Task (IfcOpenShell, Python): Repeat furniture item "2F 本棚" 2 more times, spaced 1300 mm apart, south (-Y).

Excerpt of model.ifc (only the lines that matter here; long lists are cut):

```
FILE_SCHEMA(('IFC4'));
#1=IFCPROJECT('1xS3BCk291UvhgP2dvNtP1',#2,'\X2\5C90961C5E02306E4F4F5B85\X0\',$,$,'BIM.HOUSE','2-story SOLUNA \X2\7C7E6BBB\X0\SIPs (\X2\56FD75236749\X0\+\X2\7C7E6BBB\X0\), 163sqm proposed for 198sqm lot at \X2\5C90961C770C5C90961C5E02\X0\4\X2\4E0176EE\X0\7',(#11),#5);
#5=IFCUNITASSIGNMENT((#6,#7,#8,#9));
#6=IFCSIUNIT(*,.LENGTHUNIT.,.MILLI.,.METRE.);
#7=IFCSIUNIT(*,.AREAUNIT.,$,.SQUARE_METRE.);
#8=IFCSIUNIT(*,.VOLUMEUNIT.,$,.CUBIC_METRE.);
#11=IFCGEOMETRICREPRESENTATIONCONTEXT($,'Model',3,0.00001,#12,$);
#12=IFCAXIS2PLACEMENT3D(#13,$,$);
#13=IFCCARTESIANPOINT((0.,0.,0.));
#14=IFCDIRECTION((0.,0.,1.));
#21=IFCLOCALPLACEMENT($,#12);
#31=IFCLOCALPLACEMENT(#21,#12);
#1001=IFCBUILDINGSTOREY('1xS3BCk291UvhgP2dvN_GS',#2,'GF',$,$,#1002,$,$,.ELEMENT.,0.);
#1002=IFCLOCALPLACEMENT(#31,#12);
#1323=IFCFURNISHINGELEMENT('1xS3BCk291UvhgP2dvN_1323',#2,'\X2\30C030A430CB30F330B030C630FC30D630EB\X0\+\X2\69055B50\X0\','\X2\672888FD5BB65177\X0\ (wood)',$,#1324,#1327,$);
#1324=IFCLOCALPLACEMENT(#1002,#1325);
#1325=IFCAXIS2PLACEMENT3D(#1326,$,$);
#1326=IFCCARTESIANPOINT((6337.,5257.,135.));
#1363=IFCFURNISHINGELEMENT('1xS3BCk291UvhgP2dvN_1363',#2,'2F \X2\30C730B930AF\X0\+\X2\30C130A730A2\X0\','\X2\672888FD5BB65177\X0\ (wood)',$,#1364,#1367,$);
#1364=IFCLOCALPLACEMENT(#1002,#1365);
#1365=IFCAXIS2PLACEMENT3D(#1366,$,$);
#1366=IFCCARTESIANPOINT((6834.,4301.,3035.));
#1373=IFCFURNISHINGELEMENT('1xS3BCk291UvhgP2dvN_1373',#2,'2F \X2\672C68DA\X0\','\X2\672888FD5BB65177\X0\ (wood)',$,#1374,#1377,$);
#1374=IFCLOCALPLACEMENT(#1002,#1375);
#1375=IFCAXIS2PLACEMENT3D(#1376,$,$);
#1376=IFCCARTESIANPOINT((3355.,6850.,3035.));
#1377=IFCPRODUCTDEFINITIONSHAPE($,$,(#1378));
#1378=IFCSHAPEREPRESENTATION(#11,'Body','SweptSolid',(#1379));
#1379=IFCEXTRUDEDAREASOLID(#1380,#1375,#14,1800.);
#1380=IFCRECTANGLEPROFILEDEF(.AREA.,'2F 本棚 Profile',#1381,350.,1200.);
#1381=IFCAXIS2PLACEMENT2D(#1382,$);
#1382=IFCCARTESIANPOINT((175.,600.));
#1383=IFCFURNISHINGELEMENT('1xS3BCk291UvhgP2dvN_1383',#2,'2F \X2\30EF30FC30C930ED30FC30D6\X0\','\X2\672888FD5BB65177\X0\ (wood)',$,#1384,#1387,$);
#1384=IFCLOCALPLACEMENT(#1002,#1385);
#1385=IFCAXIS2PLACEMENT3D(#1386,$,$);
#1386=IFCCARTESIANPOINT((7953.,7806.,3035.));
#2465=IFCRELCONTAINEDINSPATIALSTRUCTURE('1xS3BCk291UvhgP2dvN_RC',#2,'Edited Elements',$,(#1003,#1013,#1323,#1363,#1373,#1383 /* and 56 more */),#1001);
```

```python
import numpy as np
import ifcopenshell
import ifcopenshell.api.geometry
import ifcopenshell.api.root
import ifcopenshell.util.element
import ifcopenshell.util.placement
import ifcopenshell.util.unit

model = ifcopenshell.open("model.ifc")
unit_scale = ifcopenshell.util.unit.calculate_unit_scale(model)


def reuse_history(source, copy):
    """copy_class also copies each property set's owner history, people and application; keep the originals."""
    for rel in copy.IsDefinedBy:
        if rel.is_a("IfcRelDefinesByProperties") and (history := rel.RelatingPropertyDefinition.OwnerHistory):
            rel.RelatingPropertyDefinition.OwnerHistory = source.OwnerHistory
            ifcopenshell.util.element.remove_deep2(model, history)


source = model.by_guid("1xS3BCk291UvhgP2dvN_1373")
base = ifcopenshell.util.placement.get_local_placement(source.ObjectPlacement)
step = np.array([0.0, -1.0, 0.0]) * 1.3 / unit_scale

for i in range(1, 3):
    copy = ifcopenshell.api.root.copy_class(model, product=source)
    copy.Representation = ifcopenshell.util.element.copy_deep(
        model, source.Representation, exclude=["IfcGeometricRepresentationContext", "IfcRepresentationMap"]
    )
    reuse_history(source, copy)
    matrix = base.copy()
    matrix[:3, 3] += i * step
    print("added at", matrix[:3, 3].round(3) + 0.0)
    ifcopenshell.api.geometry.edit_object_placement(model, product=copy, matrix=matrix, is_si=False)

model.write("model_updated.ifc")
```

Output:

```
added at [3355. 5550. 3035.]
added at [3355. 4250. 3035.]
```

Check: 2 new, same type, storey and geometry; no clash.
